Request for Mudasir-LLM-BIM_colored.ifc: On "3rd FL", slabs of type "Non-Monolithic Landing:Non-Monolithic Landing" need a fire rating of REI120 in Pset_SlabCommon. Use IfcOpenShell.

First a look at what the model holds.

```python
import ifcopenshell
import ifcopenshell.util.element

model = ifcopenshell.open("Mudasir-LLM-BIM_colored.ifc")
print(model.schema)
storey = next(s for s in model.by_type("IfcBuildingStorey") if s.Name == "3rd FL")
slabs = [e for e in ifcopenshell.util.element.get_decomposition(storey) if e.is_a("IfcSlab")]
seen = {}
for e in slabs:
    element_type = ifcopenshell.util.element.get_type(e)
    key = (element_type.Name if element_type != e and element_type else None, ifcopenshell.util.element.get_pset(e, "Pset_SlabCommon", "FireRating"))
    seen[key] = seen.get(key, 0) + 1
for (name, value), count in sorted(seen.items(), key=str):
    print(count, "x", name, "|", value)
```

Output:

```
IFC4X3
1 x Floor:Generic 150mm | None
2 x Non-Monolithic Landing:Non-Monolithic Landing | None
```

```python
import ifcopenshell
import ifcopenshell.api.pset
import ifcopenshell.util.element

model = ifcopenshell.open("Mudasir-LLM-BIM_colored.ifc")

storey = next(s for s in model.by_type("IfcBuildingStorey") if s.Name == "3rd FL")
slabs = [e for e in ifcopenshell.util.element.get_decomposition(storey) if e.is_a("IfcSlab")]

count = 0
for e in slabs:
    element_type = ifcopenshell.util.element.get_type(e)
    if element_type in (None, e) or element_type.Name != "Non-Monolithic Landing:Non-Monolithic Landing":
        continue
    # add_pset returns the element's existing set when there is one.
    pset = ifcopenshell.api.pset.add_pset(model, product=e, name="Pset_SlabCommon")
    ifcopenshell.api.pset.edit_pset(model, pset=pset, properties={"FireRating": "REI120"})
    count += 1

print(count, "slabs updated")

model.write("Mudasir-LLM-BIM_colored-out.ifc")
```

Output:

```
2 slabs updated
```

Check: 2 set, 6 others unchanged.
